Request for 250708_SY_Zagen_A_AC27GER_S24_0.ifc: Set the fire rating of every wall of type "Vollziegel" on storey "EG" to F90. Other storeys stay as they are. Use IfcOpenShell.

First a look at what the model holds.

```python
import ifcopenshell
import ifcopenshell.util.element

model = ifcopenshell.open("250708_SY_Zagen_A_AC27GER_S24_0.ifc")
print(model.schema)
storey = next(s for s in model.by_type("IfcBuildingStorey") if s.Name == "EG")
walls = [e for e in ifcopenshell.util.element.get_decomposition(storey) if e.is_a("IfcWall")]
seen = {}
for e in walls:
    element_type = ifcopenshell.util.element.get_type(e)
    key = (element_type.Name if element_type != e and element_type else None, ifcopenshell.util.element.get_pset(e, "Pset_WallCommon", "FireRating"))
    seen[key] = seen.get(key, 0) + 1
for (name, value), count in sorted(seen.items(), key=str):
    print(count, "x", name, "|", value)
```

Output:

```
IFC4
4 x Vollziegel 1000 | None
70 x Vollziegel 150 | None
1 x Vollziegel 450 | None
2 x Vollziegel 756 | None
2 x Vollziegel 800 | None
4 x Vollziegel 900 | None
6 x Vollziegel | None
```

```python
import ifcopenshell
import ifcopenshell.api.pset
import ifcopenshell.util.element

model = ifcopenshell.open("250708_SY_Zagen_A_AC27GER_S24_0.ifc")

storey = next(s for s in model.by_type("IfcBuildingStorey") if s.Name == "EG")
walls = [e for e in ifcopenshell.util.element.get_decomposition(storey) if e.is_a("IfcWall")]

count = 0
for e in walls:
    element_type = ifcopenshell.util.element.get_type(e)
    if element_type in (None, e) or element_type.Name != "Vollziegel":
        continue
    # add_pset returns the element's existing set when there is one.
    pset = ifcopenshell.api.pset.add_pset(model, product=e, name="Pset_WallCommon")
    ifcopenshell.api.pset.edit_pset(model, pset=pset, properties={"FireRating": "F90"})
    count += 1

print(count, "walls updated")

model.write("250708_SY_Zagen_A_AC27GER_S24_0_edited.ifc")
```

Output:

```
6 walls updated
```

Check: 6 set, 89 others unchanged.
